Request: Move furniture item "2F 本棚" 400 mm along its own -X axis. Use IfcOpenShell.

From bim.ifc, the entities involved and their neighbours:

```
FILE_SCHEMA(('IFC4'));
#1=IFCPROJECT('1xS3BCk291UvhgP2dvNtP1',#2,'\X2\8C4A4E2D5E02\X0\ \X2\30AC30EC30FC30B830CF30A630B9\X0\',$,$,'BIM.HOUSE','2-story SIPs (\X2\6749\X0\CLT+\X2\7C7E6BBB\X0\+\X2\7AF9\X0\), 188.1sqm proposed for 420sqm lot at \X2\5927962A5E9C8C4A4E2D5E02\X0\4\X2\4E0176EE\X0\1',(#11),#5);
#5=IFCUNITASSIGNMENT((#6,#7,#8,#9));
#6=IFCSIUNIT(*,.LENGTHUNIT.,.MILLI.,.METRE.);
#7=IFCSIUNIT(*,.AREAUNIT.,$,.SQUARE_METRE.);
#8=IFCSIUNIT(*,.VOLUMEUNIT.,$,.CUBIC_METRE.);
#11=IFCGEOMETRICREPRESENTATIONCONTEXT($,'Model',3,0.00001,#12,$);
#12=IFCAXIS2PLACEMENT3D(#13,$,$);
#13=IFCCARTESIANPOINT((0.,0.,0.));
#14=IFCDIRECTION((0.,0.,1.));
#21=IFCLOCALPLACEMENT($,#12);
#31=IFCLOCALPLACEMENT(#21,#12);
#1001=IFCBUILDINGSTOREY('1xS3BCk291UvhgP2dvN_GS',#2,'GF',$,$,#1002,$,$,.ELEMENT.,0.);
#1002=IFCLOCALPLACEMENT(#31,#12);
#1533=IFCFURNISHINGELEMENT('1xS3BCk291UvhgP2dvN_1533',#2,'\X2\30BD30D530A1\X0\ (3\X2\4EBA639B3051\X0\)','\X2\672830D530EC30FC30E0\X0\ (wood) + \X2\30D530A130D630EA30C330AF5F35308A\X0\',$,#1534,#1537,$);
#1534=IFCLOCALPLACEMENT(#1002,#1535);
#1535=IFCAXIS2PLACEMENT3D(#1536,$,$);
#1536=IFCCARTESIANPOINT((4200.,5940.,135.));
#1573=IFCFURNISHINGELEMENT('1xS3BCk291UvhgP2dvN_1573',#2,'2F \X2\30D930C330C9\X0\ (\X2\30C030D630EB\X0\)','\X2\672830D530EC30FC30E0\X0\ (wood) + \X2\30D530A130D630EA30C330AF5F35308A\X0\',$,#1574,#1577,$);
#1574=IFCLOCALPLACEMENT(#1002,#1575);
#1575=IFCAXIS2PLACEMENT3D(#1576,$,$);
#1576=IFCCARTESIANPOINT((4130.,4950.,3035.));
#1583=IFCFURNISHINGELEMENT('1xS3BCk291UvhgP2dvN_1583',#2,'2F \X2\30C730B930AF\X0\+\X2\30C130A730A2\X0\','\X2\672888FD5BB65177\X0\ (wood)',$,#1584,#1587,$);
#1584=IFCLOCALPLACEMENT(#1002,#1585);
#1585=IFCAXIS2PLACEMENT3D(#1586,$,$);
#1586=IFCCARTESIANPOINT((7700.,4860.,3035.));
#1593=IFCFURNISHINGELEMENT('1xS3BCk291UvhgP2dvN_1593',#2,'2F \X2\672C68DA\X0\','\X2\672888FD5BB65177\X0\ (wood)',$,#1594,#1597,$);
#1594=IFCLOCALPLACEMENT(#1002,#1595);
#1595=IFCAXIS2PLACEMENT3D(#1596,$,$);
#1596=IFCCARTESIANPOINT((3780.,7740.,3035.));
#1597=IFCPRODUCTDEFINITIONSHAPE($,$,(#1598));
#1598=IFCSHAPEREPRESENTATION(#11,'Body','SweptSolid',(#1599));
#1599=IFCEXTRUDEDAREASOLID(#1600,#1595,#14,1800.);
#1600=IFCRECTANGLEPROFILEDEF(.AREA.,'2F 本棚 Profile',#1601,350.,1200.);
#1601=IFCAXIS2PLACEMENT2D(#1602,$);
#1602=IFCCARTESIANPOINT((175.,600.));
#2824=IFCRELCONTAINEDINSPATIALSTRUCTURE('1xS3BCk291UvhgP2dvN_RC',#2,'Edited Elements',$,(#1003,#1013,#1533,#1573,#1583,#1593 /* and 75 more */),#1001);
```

```python
import ifcopenshell
import ifcopenshell.api.geometry
import ifcopenshell.util.placement
import ifcopenshell.util.unit

model = ifcopenshell.open("bim.ifc")
unit_scale = ifcopenshell.util.unit.calculate_unit_scale(model)

item = model.by_guid("1xS3BCk291UvhgP2dvN_1593")
matrix = ifcopenshell.util.placement.get_local_placement(item.ObjectPlacement)
matrix[:3, 3] -= matrix[:3, 0] * 0.4 / unit_scale
ifcopenshell.api.geometry.edit_object_placement(model, product=item, matrix=matrix, is_si=False)

print(ifcopenshell.util.placement.get_local_placement(item.ObjectPlacement).round(3) + 0.0)

model.write("bim_edited.ifc")
```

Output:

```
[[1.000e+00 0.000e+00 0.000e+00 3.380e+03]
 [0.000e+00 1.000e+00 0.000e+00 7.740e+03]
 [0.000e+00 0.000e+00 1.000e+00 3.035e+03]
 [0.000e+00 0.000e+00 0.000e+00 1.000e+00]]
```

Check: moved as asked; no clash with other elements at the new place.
